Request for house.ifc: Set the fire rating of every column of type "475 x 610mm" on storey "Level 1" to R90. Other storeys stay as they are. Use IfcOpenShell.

First a look at what the model holds.

```python
import ifcopenshell
import ifcopenshell.util.element

model = ifcopenshell.open("house.ifc")
print(model.schema)
storey = next(s for s in model.by_type("IfcBuildingStorey") if s.Name == "Level 1")
columns = [e for e in ifcopenshell.util.element.get_decomposition(storey) if e.is_a("IfcColumn")]
seen = {}
for e in columns:
    element_type = ifcopenshell.util.element.get_type(e)
    key = (element_type.Name if element_type != e and element_type else None, ifcopenshell.util.element.get_pset(e, "Pset_ColumnCommon", "FireRating"))
    seen[key] = seen.get(key, 0) + 1
for (name, value), count in sorted(seen.items(), key=str):
    print(count, "x", name, "|", value)
```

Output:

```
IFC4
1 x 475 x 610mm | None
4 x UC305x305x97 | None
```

```python
import ifcopenshell
import ifcopenshell.api.pset
import ifcopenshell.util.element

model = ifcopenshell.open("house.ifc")

storey = next(s for s in model.by_type("IfcBuildingStorey") if s.Name == "Level 1")
columns = [e for e in ifcopenshell.util.element.get_decomposition(storey) if e.is_a("IfcColumn")]

count = 0
for e in columns:
    element_type = ifcopenshell.util.element.get_type(e)
    if element_type in (None, e) or element_type.Name != "475 x 610mm":
        continue
    # add_pset returns the element's existing set when there is one.
    pset = ifcopenshell.api.pset.add_pset(model, product=e, name="Pset_ColumnCommon")
    ifcopenshell.api.pset.edit_pset(model, pset=pset, properties={"FireRating": "R90"})
    count += 1

print(count, "columns updated")

model.write("house_edited.ifc")
```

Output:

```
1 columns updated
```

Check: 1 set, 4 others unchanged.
